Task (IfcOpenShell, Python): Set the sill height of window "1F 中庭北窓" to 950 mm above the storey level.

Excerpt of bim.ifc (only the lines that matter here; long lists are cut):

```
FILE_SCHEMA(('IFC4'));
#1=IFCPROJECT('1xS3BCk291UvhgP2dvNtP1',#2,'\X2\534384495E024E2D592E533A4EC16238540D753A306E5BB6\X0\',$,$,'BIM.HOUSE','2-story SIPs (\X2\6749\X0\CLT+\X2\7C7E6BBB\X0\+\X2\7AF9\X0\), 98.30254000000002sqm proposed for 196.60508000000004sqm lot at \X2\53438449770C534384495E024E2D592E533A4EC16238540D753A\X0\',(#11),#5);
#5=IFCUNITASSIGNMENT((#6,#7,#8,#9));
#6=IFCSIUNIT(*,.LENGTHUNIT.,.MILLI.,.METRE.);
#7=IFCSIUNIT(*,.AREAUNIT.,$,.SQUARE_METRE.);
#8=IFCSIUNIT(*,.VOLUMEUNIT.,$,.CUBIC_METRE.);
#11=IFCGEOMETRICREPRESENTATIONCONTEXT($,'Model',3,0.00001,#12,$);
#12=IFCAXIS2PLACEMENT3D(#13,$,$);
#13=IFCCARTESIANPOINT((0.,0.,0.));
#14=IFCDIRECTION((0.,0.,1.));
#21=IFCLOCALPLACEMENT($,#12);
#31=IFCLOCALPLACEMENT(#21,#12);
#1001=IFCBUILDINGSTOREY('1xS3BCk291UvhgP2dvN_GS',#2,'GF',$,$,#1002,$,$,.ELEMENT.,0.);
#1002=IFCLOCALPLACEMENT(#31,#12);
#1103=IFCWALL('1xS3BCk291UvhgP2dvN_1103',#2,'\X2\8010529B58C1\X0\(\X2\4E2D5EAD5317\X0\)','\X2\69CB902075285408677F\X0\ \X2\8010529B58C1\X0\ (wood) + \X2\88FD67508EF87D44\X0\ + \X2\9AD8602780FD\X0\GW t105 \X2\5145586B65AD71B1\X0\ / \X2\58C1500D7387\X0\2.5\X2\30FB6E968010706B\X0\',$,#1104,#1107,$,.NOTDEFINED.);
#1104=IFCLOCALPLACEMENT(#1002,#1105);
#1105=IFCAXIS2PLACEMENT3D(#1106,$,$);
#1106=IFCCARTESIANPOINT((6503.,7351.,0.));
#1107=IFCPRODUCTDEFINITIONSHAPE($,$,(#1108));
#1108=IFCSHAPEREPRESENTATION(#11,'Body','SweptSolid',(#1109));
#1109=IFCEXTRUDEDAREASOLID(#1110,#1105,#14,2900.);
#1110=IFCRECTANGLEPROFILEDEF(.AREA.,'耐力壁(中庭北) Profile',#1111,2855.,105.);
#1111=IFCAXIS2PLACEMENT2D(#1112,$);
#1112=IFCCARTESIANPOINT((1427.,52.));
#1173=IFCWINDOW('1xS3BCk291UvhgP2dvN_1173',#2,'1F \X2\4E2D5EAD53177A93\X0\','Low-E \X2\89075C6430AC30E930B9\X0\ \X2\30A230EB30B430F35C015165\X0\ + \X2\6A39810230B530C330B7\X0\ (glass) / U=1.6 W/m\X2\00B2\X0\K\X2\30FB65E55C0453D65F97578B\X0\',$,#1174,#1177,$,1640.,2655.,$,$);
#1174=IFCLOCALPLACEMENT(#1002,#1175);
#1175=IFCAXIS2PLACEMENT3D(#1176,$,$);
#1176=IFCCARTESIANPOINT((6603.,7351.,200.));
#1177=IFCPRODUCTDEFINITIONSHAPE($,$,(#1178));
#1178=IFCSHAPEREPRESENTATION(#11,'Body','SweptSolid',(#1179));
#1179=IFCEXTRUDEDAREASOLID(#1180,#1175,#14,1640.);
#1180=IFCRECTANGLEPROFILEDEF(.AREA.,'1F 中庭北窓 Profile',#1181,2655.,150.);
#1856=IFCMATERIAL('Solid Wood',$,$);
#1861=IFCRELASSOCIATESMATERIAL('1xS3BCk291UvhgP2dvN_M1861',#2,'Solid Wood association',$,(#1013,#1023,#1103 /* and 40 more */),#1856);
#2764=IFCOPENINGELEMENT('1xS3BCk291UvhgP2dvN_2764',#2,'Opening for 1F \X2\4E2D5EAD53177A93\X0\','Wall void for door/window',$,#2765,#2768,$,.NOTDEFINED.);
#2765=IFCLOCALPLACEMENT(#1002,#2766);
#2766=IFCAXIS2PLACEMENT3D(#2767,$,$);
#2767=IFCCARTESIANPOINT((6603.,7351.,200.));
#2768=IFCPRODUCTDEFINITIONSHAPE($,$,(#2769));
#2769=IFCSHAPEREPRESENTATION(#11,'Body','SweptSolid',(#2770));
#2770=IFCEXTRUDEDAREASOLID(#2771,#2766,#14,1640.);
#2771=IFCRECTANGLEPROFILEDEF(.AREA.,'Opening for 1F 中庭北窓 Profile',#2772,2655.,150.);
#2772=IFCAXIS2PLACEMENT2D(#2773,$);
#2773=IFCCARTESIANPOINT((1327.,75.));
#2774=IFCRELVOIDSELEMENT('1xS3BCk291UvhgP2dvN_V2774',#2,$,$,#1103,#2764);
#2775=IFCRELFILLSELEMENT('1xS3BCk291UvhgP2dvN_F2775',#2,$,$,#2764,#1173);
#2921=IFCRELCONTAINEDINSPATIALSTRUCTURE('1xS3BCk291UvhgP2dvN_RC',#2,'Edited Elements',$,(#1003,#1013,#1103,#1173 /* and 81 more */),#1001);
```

```python
import numpy as np
import ifcopenshell
import ifcopenshell.api.geometry
import ifcopenshell.geom
import ifcopenshell.util.element
import ifcopenshell.util.placement
import ifcopenshell.util.shape
import ifcopenshell.util.unit

model = ifcopenshell.open("bim.ifc")
unit_scale = ifcopenshell.util.unit.calculate_unit_scale(model)

window = model.by_guid("1xS3BCk291UvhgP2dvN_1173")
opening = window.FillsVoids[0].RelatingOpeningElement
storey = ifcopenshell.util.element.get_container(window, ifc_class="IfcBuildingStorey")
level = ifcopenshell.util.placement.get_local_placement(storey.ObjectPlacement)[2, 3]

# The opening's origin need not be at the sill, so measure its lowest point.
shape = ifcopenshell.geom.create_shape(ifcopenshell.geom.settings(), opening)
bottom = ifcopenshell.util.shape.get_shape_bottom_elevation(shape, shape.geometry) / unit_scale
dz = level + 0.95 / unit_scale - bottom

shift = np.array([0.0, 0.0, dz])
# The window is not placed relative to its opening, so move both.
for product in (opening, window):
    matrix = ifcopenshell.util.placement.get_local_placement(product.ObjectPlacement)
    matrix[:3, 3] += shift
    ifcopenshell.api.geometry.edit_object_placement(model, product=product, matrix=matrix, is_si=False)

print(f"moved by {dz * unit_scale:+.3f} m")

model.write("bim_rev.ifc")
```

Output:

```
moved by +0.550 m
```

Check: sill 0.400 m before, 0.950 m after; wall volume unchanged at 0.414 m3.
